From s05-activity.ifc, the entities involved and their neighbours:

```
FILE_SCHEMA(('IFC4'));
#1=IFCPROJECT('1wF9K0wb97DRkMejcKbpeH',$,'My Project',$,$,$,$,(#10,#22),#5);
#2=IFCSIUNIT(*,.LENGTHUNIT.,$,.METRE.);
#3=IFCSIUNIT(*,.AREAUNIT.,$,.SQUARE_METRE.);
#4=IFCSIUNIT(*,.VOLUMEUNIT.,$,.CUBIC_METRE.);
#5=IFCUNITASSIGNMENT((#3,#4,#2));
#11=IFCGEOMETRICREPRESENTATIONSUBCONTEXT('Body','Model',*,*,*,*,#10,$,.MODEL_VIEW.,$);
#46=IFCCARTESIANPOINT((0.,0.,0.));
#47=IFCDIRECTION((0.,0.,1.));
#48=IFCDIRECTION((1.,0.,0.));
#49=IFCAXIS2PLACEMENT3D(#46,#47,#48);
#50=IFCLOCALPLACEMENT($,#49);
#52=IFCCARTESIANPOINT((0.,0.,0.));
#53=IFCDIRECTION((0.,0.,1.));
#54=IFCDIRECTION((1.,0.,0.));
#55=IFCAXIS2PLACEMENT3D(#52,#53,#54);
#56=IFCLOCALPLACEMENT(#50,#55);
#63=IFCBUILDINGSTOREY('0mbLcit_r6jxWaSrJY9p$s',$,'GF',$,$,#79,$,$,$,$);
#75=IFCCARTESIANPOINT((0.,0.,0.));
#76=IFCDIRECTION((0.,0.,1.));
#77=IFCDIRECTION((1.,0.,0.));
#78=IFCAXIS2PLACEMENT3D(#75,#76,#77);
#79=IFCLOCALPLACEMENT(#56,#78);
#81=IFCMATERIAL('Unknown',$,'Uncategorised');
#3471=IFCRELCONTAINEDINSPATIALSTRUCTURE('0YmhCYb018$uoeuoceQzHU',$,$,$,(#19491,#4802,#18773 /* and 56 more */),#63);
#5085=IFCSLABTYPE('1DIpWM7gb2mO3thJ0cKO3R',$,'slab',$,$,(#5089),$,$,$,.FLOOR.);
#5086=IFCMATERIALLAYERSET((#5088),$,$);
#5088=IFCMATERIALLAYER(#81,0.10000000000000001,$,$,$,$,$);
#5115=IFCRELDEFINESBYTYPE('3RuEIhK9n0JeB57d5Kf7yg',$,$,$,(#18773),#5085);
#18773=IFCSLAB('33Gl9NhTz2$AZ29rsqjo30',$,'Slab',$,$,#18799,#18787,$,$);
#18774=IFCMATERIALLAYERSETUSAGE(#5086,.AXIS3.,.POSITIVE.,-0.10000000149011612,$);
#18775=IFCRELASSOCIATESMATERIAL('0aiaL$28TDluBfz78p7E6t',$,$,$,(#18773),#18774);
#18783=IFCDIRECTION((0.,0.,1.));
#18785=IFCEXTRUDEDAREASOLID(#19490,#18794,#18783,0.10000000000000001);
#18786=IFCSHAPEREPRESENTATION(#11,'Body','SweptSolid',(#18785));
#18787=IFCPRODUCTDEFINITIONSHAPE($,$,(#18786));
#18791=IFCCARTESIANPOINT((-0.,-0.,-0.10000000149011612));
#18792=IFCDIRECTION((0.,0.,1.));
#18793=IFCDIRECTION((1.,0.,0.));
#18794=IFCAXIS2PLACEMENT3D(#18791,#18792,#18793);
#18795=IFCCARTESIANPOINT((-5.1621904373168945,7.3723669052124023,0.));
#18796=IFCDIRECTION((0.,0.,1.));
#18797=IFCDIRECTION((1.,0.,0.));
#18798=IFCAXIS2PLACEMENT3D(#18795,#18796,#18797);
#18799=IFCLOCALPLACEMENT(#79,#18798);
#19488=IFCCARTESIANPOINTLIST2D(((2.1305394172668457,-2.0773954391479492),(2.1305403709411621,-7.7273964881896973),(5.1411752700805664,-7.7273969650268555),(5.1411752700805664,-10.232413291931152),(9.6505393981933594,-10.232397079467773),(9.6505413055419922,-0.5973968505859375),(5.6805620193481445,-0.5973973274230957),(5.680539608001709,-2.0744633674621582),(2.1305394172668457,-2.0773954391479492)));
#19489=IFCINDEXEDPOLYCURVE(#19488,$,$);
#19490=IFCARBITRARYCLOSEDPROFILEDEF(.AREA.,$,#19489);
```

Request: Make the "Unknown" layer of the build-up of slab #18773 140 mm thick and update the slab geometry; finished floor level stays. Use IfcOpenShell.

```python
import ifcopenshell
import ifcopenshell.util.element
import ifcopenshell.util.representation
import ifcopenshell.util.unit

model = ifcopenshell.open("s05-activity.ifc")
unit_scale = ifcopenshell.util.unit.calculate_unit_scale(model)

layer_set = model.by_id(5086)
layer = next(l for l in layer_set.MaterialLayers if l.Material and l.Material.Name == "Unknown")
change = 0.14 / unit_scale - layer.LayerThickness
layer.LayerThickness += change

# Geometry does not follow the layer set by itself.
slabs = [e for e in ifcopenshell.util.element.get_elements_by_material(model, layer_set) if e.is_a("IfcSlab")]
for slab in sorted(slabs, key=lambda e: e.id()):
    body = ifcopenshell.util.representation.get_representation(slab, "Model", "Body")
    solid = body.Items[0]
    old_depth = solid.Depth
    solid.Depth += change
    # Extruded upwards: lower the start of the extrusion so the top stays.
    x, y, z = solid.Position.Location.Coordinates
    solid.Position.Location = model.createIfcCartesianPoint((x, y, z - change))
    print(slab.id(), f"{old_depth:g} -> {solid.Depth:g}")

# The layers are counted up from the underside, which has moved.
for usage in {ifcopenshell.util.element.get_material(slab) for slab in slabs}:
    usage.OffsetFromReferenceLine -= change

model.write("s05-activity_v2.ifc")
```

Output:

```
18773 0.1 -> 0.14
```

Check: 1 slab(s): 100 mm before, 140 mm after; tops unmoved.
